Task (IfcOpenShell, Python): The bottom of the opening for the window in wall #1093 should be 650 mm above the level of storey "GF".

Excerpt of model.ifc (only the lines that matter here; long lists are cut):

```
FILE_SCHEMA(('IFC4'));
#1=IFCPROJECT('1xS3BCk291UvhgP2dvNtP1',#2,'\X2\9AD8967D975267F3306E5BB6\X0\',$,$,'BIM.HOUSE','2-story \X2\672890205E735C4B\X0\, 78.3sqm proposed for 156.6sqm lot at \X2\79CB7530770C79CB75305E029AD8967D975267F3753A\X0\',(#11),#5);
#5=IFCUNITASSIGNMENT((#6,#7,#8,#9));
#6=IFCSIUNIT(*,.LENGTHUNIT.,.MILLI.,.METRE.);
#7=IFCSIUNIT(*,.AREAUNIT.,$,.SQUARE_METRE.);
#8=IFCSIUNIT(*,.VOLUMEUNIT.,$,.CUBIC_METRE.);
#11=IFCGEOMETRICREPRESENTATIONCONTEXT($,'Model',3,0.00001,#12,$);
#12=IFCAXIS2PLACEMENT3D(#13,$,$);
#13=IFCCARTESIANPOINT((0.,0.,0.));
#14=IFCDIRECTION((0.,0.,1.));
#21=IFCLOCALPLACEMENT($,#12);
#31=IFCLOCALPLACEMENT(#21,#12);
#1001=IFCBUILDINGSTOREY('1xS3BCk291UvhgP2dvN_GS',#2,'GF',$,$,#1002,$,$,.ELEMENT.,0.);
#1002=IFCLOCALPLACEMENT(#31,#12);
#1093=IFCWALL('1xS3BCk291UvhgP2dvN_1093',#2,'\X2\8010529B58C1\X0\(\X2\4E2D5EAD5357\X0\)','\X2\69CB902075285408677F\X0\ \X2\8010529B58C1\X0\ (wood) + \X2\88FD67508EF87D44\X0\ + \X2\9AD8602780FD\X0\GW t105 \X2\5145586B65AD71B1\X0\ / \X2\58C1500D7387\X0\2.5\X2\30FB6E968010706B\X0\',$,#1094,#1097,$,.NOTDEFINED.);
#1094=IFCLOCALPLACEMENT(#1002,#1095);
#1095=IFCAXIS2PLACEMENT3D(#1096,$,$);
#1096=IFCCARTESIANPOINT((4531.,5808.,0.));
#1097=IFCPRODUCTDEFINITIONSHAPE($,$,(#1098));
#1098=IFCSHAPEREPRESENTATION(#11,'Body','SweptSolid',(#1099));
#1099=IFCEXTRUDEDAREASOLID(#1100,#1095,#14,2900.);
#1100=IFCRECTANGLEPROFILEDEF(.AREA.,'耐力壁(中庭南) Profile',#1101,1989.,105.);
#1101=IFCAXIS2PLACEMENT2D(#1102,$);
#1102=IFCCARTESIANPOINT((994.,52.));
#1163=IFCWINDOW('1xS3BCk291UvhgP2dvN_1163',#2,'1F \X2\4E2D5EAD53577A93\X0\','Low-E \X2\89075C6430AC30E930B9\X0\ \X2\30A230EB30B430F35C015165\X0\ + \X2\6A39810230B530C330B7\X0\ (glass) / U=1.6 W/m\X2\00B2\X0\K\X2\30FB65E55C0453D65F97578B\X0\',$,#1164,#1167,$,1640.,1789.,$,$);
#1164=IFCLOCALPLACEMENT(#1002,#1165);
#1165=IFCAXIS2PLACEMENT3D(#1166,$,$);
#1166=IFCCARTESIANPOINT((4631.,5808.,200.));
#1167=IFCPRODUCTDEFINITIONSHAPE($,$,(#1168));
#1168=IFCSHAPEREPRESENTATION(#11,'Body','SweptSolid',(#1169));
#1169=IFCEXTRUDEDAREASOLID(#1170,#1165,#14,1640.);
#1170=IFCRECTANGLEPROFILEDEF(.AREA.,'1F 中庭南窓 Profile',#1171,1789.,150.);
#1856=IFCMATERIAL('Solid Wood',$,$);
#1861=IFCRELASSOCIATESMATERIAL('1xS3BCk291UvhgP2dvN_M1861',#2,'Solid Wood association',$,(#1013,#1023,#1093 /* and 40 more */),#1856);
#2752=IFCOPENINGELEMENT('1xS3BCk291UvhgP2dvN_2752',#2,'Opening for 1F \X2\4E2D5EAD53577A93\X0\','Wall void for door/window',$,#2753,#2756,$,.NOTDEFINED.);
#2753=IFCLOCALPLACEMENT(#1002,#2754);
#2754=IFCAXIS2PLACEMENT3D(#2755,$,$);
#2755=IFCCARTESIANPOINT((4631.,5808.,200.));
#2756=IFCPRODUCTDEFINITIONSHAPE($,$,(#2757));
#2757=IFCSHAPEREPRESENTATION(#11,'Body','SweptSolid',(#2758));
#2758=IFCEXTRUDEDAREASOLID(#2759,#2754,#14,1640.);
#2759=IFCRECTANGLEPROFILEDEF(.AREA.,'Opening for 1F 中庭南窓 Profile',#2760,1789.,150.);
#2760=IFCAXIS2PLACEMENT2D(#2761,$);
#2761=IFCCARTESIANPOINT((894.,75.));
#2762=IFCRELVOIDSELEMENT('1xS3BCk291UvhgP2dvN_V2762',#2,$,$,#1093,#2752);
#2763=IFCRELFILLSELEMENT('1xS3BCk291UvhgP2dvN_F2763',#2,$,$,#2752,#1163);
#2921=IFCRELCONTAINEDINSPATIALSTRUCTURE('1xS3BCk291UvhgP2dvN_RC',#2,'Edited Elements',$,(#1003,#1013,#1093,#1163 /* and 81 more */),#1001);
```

```python
import numpy as np
import ifcopenshell
import ifcopenshell.api.geometry
import ifcopenshell.geom
import ifcopenshell.util.element
import ifcopenshell.util.placement
import ifcopenshell.util.shape
import ifcopenshell.util.unit

model = ifcopenshell.open("model.ifc")
unit_scale = ifcopenshell.util.unit.calculate_unit_scale(model)

window = model.by_guid("1xS3BCk291UvhgP2dvN_1163")
opening = window.FillsVoids[0].RelatingOpeningElement
storey = ifcopenshell.util.element.get_container(window, ifc_class="IfcBuildingStorey")
level = ifcopenshell.util.placement.get_local_placement(storey.ObjectPlacement)[2, 3]

# The opening's origin need not be at the sill, so measure its lowest point.
shape = ifcopenshell.geom.create_shape(ifcopenshell.geom.settings(), opening)
bottom = ifcopenshell.util.shape.get_shape_bottom_elevation(shape, shape.geometry) / unit_scale
dz = level + 650.0 - bottom

shift = np.array([0.0, 0.0, dz])
# The window is not placed relative to its opening, so move both.
for product in (opening, window):
    matrix = ifcopenshell.util.placement.get_local_placement(product.ObjectPlacement)
    matrix[:3, 3] += shift
    ifcopenshell.api.geometry.edit_object_placement(model, product=product, matrix=matrix, is_si=False)

print(f"moved by {dz * unit_scale:+.3f} m")

model.write("model_rev.ifc")
```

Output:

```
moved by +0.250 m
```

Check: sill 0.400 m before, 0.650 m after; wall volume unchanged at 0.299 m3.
